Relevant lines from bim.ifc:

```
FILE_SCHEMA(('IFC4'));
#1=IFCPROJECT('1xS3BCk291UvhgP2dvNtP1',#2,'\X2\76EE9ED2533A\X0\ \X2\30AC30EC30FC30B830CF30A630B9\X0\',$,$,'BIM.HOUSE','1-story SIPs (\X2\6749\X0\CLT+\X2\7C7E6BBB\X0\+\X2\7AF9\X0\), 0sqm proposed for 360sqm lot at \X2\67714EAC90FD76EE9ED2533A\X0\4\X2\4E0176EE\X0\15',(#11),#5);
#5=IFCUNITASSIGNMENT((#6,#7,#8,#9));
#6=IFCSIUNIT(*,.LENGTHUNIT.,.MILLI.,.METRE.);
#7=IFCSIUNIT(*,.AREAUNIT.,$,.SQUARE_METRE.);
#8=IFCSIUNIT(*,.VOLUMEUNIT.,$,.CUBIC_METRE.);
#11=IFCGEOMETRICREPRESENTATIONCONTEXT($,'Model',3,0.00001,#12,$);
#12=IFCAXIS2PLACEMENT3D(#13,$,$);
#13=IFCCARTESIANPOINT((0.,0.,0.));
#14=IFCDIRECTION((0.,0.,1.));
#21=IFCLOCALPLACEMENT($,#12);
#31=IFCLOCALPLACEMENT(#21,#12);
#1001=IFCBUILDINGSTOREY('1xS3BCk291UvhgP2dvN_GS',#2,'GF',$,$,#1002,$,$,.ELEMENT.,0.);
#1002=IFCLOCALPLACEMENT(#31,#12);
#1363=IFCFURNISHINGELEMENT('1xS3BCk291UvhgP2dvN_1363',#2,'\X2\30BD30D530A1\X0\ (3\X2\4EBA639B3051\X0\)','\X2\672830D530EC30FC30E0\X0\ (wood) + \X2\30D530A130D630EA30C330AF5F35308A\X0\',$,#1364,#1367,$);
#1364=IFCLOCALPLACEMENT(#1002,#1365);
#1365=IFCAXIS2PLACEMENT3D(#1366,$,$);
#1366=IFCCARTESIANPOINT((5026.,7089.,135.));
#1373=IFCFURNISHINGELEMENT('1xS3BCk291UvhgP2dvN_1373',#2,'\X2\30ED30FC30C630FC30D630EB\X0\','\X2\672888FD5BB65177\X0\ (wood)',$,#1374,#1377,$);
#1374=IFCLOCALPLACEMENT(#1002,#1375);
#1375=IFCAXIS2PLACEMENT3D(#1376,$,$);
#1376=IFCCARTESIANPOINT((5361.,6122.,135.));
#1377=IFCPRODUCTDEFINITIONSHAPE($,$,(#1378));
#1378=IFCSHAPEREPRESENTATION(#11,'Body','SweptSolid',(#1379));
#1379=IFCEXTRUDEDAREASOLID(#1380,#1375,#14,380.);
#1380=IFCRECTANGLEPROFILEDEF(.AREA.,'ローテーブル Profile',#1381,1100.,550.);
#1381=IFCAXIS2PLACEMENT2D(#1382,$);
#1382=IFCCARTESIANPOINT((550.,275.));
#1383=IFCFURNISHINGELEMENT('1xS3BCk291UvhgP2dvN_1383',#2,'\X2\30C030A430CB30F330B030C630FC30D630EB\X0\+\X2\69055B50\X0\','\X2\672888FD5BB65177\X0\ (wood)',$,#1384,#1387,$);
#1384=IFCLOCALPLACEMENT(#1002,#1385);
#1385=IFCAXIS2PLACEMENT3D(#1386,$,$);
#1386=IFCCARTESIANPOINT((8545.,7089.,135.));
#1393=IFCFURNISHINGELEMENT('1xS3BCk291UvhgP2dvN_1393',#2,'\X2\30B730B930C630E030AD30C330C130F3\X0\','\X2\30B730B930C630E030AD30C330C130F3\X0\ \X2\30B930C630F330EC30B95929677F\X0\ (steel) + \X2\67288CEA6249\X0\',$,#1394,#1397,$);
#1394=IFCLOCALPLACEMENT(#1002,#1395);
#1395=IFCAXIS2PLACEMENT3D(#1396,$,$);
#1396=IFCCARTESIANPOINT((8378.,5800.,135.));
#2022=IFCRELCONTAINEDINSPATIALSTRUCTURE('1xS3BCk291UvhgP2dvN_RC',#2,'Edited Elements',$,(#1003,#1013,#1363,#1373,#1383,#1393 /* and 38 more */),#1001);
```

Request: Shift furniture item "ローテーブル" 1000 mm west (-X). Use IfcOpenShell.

```python
import ifcopenshell
import ifcopenshell.api.geometry
import ifcopenshell.util.placement

model = ifcopenshell.open("bim.ifc")

item = model.by_guid("1xS3BCk291UvhgP2dvN_1373")
matrix = ifcopenshell.util.placement.get_local_placement(item.ObjectPlacement)
matrix[0, 3] -= 1000.0
ifcopenshell.api.geometry.edit_object_placement(model, product=item, matrix=matrix, is_si=False)

print(ifcopenshell.util.placement.get_local_placement(item.ObjectPlacement).round(3) + 0.0)

model.write("bim_v2.ifc")
```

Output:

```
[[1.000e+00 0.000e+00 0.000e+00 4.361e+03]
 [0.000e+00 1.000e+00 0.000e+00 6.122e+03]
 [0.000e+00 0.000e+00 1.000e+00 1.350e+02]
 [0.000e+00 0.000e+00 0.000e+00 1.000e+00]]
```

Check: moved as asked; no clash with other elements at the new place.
